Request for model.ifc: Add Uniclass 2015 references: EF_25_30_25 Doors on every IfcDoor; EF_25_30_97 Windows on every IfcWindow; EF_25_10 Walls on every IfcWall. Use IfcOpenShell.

First a look at what the model holds.

```python
import ifcopenshell

model = ifcopenshell.open("model.ifc")
print(model.schema)
print("classifications:", [c.Name for c in model.by_type("IfcClassification")])
for ifc_class in ("IfcDoor", "IfcRoof", "IfcStair", "IfcWall", "IfcWindow"):
    print(ifc_class, len(model.by_type(ifc_class)))
```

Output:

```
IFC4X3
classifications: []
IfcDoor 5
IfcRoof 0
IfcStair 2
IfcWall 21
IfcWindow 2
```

```python
import ifcopenshell
import ifcopenshell.api.classification

model = ifcopenshell.open("model.ifc")

system = ifcopenshell.api.classification.add_classification(model, classification="Uniclass 2015")

codes = {
    "IfcDoor": ("EF_25_30_25", "Doors"),
    "IfcWindow": ("EF_25_30_97", "Windows"),
    "IfcWall": ("EF_25_10", "Walls"),
}
for ifc_class, (code, name) in codes.items():
    products = model.by_type(ifc_class)
    ifcopenshell.api.classification.add_reference(
        model, products=products, classification=system, identification=code, name=name
    )
    print(code, len(products))

model.write("model_updated.ifc")
```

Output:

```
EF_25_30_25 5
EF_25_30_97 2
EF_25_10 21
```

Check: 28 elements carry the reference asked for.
